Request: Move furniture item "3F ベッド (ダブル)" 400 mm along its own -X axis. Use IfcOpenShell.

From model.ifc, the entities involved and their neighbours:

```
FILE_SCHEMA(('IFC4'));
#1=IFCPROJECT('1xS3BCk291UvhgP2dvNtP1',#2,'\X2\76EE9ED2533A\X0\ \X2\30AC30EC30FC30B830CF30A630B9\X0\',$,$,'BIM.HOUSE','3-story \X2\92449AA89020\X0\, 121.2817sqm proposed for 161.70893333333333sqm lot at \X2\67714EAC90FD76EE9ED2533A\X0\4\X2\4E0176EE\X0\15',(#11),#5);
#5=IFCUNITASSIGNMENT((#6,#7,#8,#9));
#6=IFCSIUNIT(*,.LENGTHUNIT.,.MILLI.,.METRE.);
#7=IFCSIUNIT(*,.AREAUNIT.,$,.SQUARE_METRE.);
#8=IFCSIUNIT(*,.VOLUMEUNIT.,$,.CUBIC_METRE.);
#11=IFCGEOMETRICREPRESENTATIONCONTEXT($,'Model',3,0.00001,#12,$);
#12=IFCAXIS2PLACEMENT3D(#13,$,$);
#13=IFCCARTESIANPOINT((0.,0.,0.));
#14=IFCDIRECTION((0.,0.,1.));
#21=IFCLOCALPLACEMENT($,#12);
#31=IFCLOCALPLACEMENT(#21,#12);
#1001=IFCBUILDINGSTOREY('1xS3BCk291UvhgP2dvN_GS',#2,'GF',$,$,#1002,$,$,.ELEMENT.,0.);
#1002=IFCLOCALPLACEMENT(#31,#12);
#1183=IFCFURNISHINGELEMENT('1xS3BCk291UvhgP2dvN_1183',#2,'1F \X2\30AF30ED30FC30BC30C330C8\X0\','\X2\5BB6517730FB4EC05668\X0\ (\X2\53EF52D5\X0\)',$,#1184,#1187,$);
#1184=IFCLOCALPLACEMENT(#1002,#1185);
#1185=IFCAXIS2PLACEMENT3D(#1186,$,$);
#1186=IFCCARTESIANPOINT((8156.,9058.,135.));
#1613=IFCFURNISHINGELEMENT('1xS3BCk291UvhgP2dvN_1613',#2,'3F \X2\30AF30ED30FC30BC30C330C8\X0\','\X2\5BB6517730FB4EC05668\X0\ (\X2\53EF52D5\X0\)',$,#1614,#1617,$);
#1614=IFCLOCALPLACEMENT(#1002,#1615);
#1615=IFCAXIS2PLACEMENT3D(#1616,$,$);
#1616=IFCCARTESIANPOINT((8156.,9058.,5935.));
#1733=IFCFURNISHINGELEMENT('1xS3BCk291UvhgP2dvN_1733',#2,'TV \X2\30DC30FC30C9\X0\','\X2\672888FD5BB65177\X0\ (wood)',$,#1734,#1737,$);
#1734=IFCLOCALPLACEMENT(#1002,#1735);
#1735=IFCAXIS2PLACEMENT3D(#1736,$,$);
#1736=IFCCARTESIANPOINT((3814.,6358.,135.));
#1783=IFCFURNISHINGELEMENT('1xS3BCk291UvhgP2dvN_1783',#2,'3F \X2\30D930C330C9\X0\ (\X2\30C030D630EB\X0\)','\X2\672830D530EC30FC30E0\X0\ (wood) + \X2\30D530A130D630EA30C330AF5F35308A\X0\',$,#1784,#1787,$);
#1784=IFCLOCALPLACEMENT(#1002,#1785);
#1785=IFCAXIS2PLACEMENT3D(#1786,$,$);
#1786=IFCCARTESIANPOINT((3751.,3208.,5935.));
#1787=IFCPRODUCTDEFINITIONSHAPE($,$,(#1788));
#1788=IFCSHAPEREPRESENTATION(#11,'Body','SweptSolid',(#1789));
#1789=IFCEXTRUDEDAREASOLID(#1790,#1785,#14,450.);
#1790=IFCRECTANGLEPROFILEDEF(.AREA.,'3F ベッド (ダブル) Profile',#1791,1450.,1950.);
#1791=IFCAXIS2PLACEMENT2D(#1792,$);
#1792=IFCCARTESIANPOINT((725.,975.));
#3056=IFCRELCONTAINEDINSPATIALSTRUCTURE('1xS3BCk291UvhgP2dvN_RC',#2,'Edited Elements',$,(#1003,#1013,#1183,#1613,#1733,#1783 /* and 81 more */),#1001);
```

```python
import ifcopenshell
import ifcopenshell.api.geometry
import ifcopenshell.util.placement

model = ifcopenshell.open("model.ifc")

item = model.by_id(1783)
matrix = ifcopenshell.util.placement.get_local_placement(item.ObjectPlacement)
matrix[:3, 3] -= matrix[:3, 0] * 400.0
ifcopenshell.api.geometry.edit_object_placement(model, product=item, matrix=matrix, is_si=False)

print(ifcopenshell.util.placement.get_local_placement(item.ObjectPlacement).round(3) + 0.0)

model.write("model_rev.ifc")
```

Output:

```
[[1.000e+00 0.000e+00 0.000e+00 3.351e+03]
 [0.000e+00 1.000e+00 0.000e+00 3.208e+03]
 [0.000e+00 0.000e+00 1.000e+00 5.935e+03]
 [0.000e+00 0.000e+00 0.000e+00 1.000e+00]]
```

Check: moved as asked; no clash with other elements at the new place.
